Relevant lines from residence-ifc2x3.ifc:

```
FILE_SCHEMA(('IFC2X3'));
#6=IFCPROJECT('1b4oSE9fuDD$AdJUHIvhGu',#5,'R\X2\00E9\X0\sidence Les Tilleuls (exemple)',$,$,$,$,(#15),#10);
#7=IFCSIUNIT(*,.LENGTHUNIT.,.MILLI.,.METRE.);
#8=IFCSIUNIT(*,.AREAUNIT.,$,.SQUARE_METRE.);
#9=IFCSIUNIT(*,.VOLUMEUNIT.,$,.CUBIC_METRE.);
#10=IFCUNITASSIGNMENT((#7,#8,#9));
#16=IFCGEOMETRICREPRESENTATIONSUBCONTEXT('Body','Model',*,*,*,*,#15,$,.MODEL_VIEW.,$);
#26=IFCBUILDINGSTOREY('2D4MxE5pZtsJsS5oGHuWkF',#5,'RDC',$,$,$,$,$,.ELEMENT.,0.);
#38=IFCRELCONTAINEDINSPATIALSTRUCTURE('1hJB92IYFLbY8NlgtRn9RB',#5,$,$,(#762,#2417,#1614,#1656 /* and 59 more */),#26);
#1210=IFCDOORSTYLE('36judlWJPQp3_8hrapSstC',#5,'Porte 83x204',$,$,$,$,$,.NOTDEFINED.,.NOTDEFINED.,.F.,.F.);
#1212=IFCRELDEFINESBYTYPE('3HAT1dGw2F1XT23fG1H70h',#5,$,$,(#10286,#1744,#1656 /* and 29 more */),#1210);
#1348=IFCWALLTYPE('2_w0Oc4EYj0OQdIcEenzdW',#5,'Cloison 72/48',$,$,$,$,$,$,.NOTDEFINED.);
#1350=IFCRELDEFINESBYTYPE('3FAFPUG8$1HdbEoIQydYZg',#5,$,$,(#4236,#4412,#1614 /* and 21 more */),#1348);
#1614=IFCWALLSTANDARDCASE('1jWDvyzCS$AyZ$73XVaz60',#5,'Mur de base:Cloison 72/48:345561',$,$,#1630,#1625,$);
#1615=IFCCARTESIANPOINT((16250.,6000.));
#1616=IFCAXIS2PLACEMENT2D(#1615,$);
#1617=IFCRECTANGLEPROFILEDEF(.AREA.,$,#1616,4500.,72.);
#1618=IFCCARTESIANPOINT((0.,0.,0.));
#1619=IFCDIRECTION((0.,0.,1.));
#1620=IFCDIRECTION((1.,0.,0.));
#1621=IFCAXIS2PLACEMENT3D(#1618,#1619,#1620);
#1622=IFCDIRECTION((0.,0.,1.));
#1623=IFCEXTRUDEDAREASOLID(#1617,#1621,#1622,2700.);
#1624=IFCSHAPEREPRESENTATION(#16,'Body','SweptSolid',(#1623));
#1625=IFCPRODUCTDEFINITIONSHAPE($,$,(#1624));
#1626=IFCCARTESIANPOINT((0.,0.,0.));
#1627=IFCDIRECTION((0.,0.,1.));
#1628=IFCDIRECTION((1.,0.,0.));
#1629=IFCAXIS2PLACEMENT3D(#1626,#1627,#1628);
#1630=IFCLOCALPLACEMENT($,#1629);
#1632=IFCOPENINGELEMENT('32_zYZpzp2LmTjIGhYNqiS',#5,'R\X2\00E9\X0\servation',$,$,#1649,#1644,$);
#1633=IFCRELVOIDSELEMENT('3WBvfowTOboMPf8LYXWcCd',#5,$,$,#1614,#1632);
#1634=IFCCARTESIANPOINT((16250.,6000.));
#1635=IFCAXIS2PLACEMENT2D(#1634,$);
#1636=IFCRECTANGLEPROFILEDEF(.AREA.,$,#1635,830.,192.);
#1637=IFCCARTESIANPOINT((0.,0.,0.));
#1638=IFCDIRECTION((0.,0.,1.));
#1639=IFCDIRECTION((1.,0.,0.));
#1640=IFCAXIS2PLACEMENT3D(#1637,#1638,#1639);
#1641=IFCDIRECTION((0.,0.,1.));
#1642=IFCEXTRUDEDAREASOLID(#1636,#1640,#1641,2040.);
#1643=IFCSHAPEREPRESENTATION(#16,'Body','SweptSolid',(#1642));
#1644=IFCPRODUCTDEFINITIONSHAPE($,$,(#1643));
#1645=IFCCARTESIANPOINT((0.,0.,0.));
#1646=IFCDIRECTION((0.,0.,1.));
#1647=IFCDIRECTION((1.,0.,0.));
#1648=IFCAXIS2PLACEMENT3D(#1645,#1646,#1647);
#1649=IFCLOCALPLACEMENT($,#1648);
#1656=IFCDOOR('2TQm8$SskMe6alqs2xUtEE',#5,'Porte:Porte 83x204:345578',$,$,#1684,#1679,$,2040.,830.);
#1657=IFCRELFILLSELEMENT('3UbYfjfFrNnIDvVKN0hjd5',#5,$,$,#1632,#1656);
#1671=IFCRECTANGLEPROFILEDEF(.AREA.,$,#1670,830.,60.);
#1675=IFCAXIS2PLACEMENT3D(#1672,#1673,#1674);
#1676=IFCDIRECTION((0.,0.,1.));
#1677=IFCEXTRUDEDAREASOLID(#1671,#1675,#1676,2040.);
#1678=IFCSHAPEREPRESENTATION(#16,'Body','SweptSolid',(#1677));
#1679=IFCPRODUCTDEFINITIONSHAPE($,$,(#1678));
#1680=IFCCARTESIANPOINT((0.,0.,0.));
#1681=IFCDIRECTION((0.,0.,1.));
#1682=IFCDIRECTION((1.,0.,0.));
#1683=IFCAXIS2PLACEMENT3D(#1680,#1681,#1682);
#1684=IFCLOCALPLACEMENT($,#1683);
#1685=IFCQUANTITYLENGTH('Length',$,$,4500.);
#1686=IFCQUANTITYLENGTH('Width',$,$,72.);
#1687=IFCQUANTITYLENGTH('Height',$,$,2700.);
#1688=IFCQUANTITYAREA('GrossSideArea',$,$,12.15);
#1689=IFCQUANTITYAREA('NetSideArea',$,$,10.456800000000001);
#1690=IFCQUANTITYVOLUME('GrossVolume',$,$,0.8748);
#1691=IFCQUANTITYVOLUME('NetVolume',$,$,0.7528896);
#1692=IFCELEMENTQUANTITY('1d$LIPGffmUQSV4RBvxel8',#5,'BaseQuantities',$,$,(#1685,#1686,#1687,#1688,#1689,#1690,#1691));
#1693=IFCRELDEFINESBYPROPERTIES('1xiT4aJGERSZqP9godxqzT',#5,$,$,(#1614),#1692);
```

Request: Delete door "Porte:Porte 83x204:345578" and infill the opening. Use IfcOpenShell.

```python
import ifcopenshell
import ifcopenshell.api.feature
import ifcopenshell.api.pset
import ifcopenshell.api.root
import ifcopenshell.geom
import ifcopenshell.util.element
import ifcopenshell.util.shape
import ifcopenshell.util.unit

model = ifcopenshell.open("residence-ifc2x3.ifc")
area_scale = ifcopenshell.util.unit.calculate_unit_scale(model, "AREAUNIT")
volume_scale = ifcopenshell.util.unit.calculate_unit_scale(model, "VOLUMEUNIT")
settings = ifcopenshell.geom.settings()


def volume(element):
    """Net volume in cubic metres, openings subtracted."""
    shape = ifcopenshell.geom.create_shape(settings, element)
    return ifcopenshell.util.shape.get_volume(shape.geometry)


door = model.by_guid("2TQm8$SskMe6alqs2xUtEE")
opening = door.FillsVoids[0].RelatingOpeningElement
wall = opening.VoidsElements[0].RelatingBuildingElement
before = volume(wall)

ifcopenshell.api.root.remove_product(model, product=door)
ifcopenshell.api.feature.remove_feature(model, feature=opening)

after = volume(wall)
thickness = 0.072  # wall thickness in metres

# Update the wall's stored quantities.
qto = model.by_id(ifcopenshell.util.element.get_pset(wall, "BaseQuantities", should_inherit=False)["id"])
ifcopenshell.api.pset.edit_qto(model, qto=qto, properties={
    "NetSideArea": after / thickness / area_scale,
    "NetVolume": after / volume_scale,
})

print(f"wall volume {before:.3f} -> {after:.3f} m3")

model.write("residence-ifc2x3_edited.ifc")
```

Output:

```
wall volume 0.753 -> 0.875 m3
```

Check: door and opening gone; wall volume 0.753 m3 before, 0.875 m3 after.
